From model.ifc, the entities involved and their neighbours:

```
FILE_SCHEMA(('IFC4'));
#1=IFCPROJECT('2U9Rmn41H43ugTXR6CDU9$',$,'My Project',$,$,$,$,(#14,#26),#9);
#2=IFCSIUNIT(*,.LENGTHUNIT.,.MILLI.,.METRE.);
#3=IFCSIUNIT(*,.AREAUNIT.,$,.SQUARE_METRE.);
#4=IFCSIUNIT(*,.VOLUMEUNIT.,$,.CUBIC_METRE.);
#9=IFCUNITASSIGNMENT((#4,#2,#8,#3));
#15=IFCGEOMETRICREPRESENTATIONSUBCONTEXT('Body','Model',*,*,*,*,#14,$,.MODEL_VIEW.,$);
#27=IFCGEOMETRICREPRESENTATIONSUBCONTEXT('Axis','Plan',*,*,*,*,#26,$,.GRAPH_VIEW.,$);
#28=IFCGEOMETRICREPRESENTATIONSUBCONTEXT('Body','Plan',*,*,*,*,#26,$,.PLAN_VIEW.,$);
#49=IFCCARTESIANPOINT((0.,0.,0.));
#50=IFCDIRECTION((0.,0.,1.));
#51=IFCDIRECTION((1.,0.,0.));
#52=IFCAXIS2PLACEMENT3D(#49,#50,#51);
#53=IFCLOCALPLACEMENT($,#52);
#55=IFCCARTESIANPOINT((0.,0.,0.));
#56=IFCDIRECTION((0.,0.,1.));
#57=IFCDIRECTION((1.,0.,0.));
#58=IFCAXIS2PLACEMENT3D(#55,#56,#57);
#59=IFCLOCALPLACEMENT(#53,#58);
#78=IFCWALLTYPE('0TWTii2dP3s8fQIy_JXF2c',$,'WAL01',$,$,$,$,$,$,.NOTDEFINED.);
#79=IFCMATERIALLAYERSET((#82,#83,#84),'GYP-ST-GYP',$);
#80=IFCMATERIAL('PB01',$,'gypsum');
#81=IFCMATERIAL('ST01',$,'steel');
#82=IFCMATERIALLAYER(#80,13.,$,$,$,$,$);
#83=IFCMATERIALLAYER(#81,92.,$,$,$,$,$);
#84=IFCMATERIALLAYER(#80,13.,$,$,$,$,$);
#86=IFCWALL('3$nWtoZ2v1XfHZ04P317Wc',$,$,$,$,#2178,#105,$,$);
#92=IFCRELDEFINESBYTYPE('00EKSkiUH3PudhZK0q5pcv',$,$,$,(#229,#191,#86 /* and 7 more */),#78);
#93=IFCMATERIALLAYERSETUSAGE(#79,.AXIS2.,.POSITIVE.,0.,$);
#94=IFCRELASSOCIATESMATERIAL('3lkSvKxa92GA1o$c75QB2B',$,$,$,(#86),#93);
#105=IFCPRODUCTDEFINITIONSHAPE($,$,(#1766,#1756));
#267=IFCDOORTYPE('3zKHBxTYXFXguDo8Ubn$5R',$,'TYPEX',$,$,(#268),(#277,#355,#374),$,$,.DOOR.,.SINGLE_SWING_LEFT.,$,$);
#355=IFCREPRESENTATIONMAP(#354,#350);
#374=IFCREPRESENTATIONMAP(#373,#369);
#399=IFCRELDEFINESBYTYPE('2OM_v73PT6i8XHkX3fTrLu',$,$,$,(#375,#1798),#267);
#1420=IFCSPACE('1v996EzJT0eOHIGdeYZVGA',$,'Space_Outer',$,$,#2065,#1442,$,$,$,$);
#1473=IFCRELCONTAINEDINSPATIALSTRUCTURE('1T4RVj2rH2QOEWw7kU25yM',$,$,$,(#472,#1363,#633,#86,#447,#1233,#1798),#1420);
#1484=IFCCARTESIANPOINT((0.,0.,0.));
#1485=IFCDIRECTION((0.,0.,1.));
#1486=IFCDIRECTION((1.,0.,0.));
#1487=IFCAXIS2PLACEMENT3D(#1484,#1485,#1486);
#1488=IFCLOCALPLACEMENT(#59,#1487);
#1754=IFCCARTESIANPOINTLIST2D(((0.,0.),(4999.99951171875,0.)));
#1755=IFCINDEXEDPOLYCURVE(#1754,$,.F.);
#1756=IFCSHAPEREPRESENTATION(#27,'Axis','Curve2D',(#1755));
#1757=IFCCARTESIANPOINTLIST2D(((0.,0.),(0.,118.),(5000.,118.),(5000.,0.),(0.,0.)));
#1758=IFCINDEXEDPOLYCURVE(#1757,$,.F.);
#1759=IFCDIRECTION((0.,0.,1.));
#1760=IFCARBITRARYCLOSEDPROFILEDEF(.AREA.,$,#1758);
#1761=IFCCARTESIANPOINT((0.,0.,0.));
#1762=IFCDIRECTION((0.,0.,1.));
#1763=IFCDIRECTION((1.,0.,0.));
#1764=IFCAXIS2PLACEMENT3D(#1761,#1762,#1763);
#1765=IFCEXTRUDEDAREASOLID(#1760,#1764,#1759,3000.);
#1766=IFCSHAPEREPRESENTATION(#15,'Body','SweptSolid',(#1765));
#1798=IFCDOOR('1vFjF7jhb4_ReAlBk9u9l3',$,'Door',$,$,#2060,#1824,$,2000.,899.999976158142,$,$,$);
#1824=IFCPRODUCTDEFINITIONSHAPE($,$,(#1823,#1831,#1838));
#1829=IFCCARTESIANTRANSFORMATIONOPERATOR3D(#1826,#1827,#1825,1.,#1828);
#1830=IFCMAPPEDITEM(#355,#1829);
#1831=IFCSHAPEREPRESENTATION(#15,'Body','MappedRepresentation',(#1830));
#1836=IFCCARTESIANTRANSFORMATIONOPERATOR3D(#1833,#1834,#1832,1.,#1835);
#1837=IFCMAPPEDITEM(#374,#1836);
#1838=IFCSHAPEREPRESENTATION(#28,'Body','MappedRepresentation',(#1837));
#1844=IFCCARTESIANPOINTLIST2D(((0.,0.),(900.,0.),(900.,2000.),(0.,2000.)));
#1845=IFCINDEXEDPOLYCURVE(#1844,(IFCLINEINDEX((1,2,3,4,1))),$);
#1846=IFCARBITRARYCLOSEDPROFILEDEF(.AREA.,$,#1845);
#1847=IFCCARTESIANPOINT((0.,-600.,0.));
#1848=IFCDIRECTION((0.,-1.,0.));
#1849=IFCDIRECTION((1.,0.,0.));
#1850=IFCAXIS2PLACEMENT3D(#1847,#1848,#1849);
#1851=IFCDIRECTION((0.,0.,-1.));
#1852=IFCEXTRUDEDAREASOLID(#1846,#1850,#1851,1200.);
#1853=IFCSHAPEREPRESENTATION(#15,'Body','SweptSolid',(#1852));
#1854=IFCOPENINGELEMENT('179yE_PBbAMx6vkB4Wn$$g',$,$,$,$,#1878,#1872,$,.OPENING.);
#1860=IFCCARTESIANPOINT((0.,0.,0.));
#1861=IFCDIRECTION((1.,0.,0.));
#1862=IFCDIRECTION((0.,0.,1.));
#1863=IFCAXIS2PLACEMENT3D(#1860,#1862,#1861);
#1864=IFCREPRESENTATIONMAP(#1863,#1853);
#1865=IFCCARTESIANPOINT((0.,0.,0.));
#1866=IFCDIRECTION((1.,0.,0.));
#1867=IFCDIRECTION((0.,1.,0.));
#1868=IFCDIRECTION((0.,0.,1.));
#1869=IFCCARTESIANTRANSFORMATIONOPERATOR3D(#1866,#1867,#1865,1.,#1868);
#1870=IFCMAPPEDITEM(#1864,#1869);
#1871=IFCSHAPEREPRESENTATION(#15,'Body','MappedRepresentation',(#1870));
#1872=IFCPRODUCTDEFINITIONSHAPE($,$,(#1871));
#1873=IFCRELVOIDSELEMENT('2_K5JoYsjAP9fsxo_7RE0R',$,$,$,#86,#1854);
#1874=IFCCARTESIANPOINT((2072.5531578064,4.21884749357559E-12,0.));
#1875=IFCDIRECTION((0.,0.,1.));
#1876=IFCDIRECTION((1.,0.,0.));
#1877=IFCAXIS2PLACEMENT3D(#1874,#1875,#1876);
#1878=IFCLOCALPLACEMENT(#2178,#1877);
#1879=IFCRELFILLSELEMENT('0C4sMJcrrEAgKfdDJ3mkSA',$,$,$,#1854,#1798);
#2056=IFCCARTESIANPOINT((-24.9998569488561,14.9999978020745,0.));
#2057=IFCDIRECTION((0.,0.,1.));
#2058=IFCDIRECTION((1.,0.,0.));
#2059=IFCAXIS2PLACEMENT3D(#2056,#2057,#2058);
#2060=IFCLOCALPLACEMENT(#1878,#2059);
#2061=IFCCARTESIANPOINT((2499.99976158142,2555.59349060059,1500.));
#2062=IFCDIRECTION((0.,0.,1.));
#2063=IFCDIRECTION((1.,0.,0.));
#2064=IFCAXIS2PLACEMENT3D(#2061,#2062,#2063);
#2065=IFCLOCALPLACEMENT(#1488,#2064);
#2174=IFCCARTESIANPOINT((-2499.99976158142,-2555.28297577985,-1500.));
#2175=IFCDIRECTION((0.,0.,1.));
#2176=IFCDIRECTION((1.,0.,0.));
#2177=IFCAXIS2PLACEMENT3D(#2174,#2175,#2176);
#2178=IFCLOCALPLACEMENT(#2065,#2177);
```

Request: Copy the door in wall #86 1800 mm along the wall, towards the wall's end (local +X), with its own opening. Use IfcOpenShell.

```python
import ifcopenshell
import ifcopenshell.api.feature
import ifcopenshell.api.geometry
import ifcopenshell.api.root
import ifcopenshell.geom
import ifcopenshell.util.element
import ifcopenshell.util.placement
import ifcopenshell.util.shape
import ifcopenshell.util.unit

model = ifcopenshell.open("model.ifc")
unit_scale = ifcopenshell.util.unit.calculate_unit_scale(model)
settings = ifcopenshell.geom.settings()


def volume(element):
    """Net volume in cubic metres, openings subtracted."""
    shape = ifcopenshell.geom.create_shape(settings, element)
    return ifcopenshell.util.shape.get_volume(shape.geometry)


door = model.by_guid("1vFjF7jhb4_ReAlBk9u9l3")
opening = door.FillsVoids[0].RelatingOpeningElement
wall = opening.VoidsElements[0].RelatingBuildingElement
before = volume(wall)
shift = ifcopenshell.util.placement.get_local_placement(wall.ObjectPlacement)[:3, 0] * 1.8 / unit_scale

# copy_class copies the void relationship, type, container and properties, but no geometry.
new_opening = ifcopenshell.api.root.copy_class(model, product=opening)
new_opening.Representation = ifcopenshell.util.element.copy_deep(
    model, opening.Representation, exclude=["IfcGeometricRepresentationContext", "IfcRepresentationMap"]
)
new_door = ifcopenshell.api.root.copy_class(model, product=door)
new_door.Representation = ifcopenshell.util.element.copy_deep(
    model, door.Representation, exclude=["IfcGeometricRepresentationContext", "IfcRepresentationMap"]
)
ifcopenshell.api.feature.add_filling(model, opening=new_opening, element=new_door)

for old, new in ((opening, new_opening), (door, new_door)):
    matrix = ifcopenshell.util.placement.get_local_placement(old.ObjectPlacement)
    matrix[:3, 3] += shift
    ifcopenshell.api.geometry.edit_object_placement(model, product=new, matrix=matrix, is_si=False)

after = volume(wall)

print(f"wall volume {before:.3f} -> {after:.3f} m3")

model.write("model_edited.ifc")
```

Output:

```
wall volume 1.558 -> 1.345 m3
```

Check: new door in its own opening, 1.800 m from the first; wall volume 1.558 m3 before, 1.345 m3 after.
